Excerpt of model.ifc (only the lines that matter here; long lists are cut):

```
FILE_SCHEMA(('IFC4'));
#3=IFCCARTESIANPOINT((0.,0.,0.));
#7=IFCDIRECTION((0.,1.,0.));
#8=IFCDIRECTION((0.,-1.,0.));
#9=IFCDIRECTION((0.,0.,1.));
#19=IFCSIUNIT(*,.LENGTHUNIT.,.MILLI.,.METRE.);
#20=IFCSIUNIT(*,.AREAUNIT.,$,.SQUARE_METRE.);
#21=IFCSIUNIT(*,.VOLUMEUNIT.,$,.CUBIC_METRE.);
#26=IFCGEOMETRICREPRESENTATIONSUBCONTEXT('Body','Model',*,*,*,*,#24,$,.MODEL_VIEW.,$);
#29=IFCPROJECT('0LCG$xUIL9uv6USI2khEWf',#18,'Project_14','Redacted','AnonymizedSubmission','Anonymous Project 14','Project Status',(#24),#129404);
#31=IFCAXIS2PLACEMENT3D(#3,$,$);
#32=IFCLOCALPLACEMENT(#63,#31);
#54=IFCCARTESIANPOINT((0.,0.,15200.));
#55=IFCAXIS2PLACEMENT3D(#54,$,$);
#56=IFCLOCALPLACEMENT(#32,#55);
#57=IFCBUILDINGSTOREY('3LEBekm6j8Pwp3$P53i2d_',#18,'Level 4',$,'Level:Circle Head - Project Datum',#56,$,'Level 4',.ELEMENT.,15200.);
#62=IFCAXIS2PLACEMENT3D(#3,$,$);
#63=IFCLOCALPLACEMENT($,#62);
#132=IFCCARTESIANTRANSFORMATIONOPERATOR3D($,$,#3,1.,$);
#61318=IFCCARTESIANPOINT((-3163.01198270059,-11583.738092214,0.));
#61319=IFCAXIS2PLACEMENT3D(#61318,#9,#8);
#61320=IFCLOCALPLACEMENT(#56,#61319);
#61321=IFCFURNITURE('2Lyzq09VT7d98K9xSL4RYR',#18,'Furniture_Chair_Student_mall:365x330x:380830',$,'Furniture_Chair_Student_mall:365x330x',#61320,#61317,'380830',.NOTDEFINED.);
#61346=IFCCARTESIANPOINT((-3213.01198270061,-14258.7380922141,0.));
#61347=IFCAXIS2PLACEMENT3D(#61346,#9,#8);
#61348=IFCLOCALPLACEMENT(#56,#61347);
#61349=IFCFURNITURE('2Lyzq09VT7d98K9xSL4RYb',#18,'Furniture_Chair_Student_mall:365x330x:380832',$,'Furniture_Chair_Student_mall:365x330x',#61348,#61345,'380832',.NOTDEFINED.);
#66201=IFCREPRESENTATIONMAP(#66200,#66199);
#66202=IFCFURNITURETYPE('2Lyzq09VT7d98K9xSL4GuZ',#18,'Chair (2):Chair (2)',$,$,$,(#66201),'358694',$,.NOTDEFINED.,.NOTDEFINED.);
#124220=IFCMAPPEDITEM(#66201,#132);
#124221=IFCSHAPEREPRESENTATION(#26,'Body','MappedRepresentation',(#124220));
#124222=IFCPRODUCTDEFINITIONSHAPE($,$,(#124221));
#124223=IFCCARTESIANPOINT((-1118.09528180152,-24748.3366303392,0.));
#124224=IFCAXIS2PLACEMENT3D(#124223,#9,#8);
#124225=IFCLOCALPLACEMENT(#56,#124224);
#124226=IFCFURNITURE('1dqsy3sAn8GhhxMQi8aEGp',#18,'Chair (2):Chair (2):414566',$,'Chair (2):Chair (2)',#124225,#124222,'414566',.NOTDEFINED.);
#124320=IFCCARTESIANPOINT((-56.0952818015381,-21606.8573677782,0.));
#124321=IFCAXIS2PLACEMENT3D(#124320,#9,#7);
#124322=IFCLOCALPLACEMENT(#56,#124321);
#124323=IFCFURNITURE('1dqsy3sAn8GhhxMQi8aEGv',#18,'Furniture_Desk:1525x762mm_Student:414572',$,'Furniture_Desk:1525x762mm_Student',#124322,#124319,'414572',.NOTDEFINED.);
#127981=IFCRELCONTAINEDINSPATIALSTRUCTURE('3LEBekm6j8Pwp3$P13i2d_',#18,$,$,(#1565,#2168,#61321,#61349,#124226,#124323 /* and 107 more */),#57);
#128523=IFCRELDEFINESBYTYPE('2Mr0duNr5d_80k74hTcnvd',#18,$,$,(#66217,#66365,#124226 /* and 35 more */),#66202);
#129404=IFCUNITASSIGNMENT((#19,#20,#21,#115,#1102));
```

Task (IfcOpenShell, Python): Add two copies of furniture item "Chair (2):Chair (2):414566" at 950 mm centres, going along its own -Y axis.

```python
import ifcopenshell
import ifcopenshell.api.geometry
import ifcopenshell.api.root
import ifcopenshell.util.element
import ifcopenshell.util.placement
import ifcopenshell.util.unit

model = ifcopenshell.open("model.ifc")
unit_scale = ifcopenshell.util.unit.calculate_unit_scale(model)


def reuse_history(source, copy):
    """copy_class also copies each property set's owner history, people and application; keep the originals."""
    for rel in copy.IsDefinedBy:
        if rel.is_a("IfcRelDefinesByProperties") and (history := rel.RelatingPropertyDefinition.OwnerHistory):
            rel.RelatingPropertyDefinition.OwnerHistory = source.OwnerHistory
            ifcopenshell.util.element.remove_deep2(model, history)


source = model.by_id(124226)
base = ifcopenshell.util.placement.get_local_placement(source.ObjectPlacement)
step = -base[:3, 1] * 0.95 / unit_scale

for i in range(1, 3):
    copy = ifcopenshell.api.root.copy_class(model, product=source)
    copy.Representation = ifcopenshell.util.element.copy_deep(
        model, source.Representation, exclude=["IfcGeometricRepresentationContext", "IfcRepresentationMap"]
    )
    copy.Name = "Chair (2):Chair (2)"
    copy.Tag = None
    reuse_history(source, copy)
    matrix = base.copy()
    matrix[:3, 3] += i * step
    print("added at", matrix[:3, 3].round(3) + 0.0)
    ifcopenshell.api.geometry.edit_object_placement(model, product=copy, matrix=matrix, is_si=False)

model.write("model_edited.ifc")
```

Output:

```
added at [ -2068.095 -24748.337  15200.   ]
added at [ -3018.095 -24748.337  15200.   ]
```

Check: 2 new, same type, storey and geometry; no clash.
